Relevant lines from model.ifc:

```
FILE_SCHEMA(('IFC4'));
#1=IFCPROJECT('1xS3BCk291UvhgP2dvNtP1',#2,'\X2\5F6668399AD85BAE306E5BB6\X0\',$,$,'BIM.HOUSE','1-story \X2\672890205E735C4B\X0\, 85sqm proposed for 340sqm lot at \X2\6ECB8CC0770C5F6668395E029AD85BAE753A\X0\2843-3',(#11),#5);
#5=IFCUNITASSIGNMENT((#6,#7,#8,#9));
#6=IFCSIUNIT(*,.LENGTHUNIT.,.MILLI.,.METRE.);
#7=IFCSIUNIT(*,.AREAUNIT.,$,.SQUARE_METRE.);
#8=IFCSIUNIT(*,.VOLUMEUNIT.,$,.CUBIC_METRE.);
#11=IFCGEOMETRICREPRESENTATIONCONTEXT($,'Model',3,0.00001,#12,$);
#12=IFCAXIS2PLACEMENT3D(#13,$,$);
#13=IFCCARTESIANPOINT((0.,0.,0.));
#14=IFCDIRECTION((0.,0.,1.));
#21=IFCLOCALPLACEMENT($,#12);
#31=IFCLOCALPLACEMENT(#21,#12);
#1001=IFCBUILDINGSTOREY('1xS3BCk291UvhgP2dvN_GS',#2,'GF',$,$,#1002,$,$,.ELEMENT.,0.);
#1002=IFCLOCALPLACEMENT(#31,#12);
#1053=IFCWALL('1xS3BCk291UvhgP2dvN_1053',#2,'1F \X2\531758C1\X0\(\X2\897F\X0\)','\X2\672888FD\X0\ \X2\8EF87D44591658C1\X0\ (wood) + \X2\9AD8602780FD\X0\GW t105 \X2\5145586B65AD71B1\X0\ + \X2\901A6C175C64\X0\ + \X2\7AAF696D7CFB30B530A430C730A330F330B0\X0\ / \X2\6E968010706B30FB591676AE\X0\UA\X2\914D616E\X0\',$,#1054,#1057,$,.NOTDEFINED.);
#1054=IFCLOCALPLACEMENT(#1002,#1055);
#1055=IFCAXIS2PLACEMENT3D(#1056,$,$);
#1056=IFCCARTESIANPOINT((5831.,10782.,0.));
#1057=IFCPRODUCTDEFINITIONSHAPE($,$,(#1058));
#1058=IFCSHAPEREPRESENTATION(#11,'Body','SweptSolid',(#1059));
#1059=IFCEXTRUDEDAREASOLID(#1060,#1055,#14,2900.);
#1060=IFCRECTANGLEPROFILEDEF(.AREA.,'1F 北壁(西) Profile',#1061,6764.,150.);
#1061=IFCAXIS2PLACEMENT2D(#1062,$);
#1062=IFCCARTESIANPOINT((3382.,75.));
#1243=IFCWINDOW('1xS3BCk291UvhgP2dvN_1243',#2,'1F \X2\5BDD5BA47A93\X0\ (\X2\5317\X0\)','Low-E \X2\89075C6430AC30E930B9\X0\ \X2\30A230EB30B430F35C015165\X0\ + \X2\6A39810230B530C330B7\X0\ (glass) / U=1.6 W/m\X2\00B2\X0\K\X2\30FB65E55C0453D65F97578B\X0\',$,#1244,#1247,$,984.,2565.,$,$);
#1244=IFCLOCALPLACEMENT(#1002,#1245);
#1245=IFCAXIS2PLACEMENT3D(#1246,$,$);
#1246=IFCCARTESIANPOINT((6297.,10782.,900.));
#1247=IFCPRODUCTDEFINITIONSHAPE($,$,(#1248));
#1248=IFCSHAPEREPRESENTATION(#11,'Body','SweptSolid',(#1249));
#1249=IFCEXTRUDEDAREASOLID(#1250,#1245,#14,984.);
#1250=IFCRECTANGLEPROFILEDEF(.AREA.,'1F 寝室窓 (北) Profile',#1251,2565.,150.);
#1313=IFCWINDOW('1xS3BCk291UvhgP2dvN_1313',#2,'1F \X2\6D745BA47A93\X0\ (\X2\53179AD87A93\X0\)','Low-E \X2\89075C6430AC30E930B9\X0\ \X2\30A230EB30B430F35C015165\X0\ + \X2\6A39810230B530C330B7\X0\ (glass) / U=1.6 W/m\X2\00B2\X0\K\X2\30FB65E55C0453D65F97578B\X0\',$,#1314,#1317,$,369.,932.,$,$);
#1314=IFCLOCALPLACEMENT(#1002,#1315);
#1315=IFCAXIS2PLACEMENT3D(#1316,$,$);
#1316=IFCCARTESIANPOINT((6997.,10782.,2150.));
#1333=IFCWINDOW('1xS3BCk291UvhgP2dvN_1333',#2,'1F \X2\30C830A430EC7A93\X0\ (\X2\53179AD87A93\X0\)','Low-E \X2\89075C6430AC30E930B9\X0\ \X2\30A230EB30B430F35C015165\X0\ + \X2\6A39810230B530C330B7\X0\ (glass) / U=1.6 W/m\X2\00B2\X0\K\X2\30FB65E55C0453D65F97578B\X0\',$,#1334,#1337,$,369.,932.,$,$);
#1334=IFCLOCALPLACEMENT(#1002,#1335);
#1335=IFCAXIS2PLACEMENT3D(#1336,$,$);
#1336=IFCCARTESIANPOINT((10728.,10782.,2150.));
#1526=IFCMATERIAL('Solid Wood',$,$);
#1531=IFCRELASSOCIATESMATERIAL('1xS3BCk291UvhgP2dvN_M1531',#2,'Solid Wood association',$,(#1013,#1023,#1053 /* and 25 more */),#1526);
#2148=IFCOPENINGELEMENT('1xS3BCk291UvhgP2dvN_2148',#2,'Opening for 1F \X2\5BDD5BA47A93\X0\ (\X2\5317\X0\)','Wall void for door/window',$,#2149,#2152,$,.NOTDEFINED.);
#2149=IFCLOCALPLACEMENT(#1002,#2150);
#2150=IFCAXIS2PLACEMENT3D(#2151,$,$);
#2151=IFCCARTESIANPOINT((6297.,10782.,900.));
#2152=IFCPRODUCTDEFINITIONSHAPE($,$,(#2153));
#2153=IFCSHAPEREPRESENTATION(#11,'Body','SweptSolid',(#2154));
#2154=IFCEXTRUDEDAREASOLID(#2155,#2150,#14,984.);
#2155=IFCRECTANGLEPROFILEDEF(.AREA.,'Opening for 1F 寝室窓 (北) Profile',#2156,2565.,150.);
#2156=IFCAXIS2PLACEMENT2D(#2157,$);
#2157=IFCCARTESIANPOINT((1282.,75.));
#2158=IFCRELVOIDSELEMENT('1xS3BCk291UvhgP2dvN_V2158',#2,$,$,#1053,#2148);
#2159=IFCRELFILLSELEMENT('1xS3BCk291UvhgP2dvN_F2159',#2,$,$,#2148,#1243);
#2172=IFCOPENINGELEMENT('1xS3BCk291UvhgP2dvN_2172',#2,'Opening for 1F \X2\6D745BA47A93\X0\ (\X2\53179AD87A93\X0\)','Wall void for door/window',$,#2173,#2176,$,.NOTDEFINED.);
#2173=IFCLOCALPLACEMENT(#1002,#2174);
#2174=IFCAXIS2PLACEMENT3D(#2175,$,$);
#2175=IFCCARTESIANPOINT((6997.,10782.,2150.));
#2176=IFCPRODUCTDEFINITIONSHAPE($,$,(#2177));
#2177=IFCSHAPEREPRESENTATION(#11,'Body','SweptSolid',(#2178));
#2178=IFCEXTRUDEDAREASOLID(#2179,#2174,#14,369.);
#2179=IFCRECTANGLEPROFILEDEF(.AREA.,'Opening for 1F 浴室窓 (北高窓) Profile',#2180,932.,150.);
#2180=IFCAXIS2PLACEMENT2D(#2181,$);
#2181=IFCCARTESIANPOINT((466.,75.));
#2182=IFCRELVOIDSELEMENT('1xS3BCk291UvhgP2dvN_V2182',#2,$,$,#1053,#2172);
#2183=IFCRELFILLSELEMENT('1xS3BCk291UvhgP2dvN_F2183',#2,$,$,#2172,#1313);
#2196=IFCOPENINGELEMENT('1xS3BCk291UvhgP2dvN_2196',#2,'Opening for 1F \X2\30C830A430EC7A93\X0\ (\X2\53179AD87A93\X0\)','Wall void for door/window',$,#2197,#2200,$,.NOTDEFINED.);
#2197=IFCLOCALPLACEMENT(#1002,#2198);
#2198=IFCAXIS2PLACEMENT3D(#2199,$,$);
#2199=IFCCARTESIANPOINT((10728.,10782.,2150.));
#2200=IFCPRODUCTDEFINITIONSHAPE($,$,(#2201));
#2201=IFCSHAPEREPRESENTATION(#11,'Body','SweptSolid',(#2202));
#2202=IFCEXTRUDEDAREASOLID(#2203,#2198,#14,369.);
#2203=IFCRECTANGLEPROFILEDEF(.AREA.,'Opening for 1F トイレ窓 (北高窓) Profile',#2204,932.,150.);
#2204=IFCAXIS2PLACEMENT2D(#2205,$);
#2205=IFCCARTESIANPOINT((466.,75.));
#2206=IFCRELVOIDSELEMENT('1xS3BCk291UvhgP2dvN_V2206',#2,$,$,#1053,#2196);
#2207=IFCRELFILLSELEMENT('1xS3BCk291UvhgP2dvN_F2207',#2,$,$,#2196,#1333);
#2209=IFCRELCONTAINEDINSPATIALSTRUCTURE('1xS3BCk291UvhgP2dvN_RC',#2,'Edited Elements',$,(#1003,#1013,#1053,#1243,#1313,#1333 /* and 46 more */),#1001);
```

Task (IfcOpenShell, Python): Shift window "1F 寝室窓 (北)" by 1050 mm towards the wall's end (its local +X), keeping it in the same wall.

```python
import ifcopenshell
import ifcopenshell.api.geometry
import ifcopenshell.util.placement

model = ifcopenshell.open("model.ifc")

window = model.by_id(1243)
opening = window.FillsVoids[0].RelatingOpeningElement
wall = opening.VoidsElements[0].RelatingBuildingElement

wall_matrix = ifcopenshell.util.placement.get_local_placement(wall.ObjectPlacement)
shift = wall_matrix[:3, 0] * 1050.0
before = ifcopenshell.util.placement.get_local_placement(window.ObjectPlacement)[:3, 3].copy()

# The window is not placed relative to its opening, so move both.
for product in (opening, window):
    matrix = ifcopenshell.util.placement.get_local_placement(product.ObjectPlacement)
    matrix[:3, 3] += shift
    ifcopenshell.api.geometry.edit_object_placement(model, product=product, matrix=matrix, is_si=False)

after = ifcopenshell.util.placement.get_local_placement(window.ObjectPlacement)[:3, 3]
print("window moved by", (after - before).round(3) + 0.0)

model.write("model_rev.ifc")
```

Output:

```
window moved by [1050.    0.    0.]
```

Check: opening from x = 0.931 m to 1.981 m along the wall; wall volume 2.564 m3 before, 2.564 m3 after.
